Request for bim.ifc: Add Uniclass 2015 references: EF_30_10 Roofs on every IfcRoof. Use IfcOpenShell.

First a look at what the model holds.

```python
import ifcopenshell

model = ifcopenshell.open("bim.ifc")
print(model.schema)
print("classifications:", [c.Name for c in model.by_type("IfcClassification")])
for ifc_class in ("IfcDoor", "IfcRoof", "IfcStair", "IfcWall", "IfcWindow"):
    print(ifc_class, len(model.by_type(ifc_class)))
```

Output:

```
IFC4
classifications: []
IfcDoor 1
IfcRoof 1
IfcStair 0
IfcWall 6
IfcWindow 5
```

```python
import ifcopenshell
import ifcopenshell.api.classification

model = ifcopenshell.open("bim.ifc")

system = ifcopenshell.api.classification.add_classification(model, classification="Uniclass 2015")

codes = {
    "IfcRoof": ("EF_30_10", "Roofs"),
}
for ifc_class, (code, name) in codes.items():
    products = model.by_type(ifc_class)
    ifcopenshell.api.classification.add_reference(
        model, products=products, classification=system, identification=code, name=name
    )
    print(code, len(products))

model.write("bim-out.ifc")
```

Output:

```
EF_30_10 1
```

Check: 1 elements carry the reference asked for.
